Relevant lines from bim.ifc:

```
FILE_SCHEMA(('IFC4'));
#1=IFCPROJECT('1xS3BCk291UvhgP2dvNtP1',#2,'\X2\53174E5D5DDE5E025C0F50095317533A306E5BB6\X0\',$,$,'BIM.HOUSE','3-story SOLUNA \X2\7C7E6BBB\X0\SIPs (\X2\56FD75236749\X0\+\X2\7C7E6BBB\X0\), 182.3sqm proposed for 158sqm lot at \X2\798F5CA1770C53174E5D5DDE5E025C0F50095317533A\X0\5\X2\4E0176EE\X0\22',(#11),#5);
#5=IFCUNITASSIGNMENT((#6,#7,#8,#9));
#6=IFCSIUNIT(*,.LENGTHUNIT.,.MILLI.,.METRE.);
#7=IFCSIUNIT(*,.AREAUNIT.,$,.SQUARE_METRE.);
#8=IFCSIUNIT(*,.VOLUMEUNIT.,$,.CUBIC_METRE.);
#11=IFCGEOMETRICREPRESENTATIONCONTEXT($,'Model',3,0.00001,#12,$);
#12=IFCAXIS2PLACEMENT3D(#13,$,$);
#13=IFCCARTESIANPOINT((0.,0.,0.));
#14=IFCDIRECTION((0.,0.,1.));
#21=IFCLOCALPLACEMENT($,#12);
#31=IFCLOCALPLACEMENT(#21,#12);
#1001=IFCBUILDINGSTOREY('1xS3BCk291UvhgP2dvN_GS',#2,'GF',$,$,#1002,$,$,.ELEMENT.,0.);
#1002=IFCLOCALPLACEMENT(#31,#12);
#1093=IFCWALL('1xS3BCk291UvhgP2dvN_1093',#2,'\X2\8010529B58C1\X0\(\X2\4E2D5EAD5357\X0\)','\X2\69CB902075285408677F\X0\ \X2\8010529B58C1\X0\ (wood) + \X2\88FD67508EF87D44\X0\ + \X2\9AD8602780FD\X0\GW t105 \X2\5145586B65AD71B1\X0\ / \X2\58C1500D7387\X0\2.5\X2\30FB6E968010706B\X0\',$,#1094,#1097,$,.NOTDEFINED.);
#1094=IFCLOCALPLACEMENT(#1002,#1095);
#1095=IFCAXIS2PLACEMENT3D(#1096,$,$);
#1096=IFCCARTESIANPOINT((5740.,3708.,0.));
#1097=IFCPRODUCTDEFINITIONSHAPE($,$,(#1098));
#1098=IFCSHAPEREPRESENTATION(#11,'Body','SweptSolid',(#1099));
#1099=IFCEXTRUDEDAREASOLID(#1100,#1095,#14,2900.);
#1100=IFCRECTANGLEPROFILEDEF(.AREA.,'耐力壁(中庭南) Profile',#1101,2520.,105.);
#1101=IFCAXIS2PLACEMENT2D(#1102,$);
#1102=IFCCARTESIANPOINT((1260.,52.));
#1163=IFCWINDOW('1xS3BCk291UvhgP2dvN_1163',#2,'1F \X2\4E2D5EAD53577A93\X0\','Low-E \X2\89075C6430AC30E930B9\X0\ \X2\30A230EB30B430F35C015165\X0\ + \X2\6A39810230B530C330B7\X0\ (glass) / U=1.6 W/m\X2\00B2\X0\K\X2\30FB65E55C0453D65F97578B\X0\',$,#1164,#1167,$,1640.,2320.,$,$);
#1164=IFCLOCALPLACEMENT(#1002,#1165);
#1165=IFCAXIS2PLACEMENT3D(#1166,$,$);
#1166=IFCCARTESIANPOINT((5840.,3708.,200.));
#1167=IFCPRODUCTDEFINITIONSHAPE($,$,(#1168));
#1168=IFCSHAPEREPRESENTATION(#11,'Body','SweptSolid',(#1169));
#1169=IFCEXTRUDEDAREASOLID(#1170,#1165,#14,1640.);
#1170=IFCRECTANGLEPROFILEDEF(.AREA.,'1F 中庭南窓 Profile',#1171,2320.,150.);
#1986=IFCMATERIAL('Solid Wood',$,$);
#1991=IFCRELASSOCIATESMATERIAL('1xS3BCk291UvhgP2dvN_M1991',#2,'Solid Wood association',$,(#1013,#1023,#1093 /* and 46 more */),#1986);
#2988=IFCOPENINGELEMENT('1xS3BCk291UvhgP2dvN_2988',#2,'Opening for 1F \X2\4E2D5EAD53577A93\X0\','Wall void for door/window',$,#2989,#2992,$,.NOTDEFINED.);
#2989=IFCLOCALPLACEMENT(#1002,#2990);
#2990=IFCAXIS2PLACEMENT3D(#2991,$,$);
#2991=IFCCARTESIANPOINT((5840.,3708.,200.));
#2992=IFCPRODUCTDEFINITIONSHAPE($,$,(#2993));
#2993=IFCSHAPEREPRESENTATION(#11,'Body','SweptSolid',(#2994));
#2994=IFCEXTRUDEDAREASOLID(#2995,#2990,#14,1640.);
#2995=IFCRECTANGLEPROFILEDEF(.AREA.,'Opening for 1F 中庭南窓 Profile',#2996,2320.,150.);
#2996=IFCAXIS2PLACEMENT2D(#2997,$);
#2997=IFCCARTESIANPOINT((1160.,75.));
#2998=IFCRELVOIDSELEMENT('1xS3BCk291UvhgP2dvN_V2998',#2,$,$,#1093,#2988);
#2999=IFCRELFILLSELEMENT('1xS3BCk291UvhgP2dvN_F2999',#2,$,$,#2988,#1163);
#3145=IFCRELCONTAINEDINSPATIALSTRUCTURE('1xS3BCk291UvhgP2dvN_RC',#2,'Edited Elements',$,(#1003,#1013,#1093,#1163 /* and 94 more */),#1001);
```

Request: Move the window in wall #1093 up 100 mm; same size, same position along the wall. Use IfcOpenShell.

```python
import numpy as np
import ifcopenshell
import ifcopenshell.api.geometry
import ifcopenshell.util.placement
import ifcopenshell.util.unit

model = ifcopenshell.open("bim.ifc")
unit_scale = ifcopenshell.util.unit.calculate_unit_scale(model)

window = model.by_guid("1xS3BCk291UvhgP2dvN_1163")
opening = window.FillsVoids[0].RelatingOpeningElement
dz = 100.0

shift = np.array([0.0, 0.0, dz])
# The window is not placed relative to its opening, so move both.
for product in (opening, window):
    matrix = ifcopenshell.util.placement.get_local_placement(product.ObjectPlacement)
    matrix[:3, 3] += shift
    ifcopenshell.api.geometry.edit_object_placement(model, product=product, matrix=matrix, is_si=False)

print(f"moved by {dz * unit_scale:+.3f} m")

model.write("bim_v2.ifc")
```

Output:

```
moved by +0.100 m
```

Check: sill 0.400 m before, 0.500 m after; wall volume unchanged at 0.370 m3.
